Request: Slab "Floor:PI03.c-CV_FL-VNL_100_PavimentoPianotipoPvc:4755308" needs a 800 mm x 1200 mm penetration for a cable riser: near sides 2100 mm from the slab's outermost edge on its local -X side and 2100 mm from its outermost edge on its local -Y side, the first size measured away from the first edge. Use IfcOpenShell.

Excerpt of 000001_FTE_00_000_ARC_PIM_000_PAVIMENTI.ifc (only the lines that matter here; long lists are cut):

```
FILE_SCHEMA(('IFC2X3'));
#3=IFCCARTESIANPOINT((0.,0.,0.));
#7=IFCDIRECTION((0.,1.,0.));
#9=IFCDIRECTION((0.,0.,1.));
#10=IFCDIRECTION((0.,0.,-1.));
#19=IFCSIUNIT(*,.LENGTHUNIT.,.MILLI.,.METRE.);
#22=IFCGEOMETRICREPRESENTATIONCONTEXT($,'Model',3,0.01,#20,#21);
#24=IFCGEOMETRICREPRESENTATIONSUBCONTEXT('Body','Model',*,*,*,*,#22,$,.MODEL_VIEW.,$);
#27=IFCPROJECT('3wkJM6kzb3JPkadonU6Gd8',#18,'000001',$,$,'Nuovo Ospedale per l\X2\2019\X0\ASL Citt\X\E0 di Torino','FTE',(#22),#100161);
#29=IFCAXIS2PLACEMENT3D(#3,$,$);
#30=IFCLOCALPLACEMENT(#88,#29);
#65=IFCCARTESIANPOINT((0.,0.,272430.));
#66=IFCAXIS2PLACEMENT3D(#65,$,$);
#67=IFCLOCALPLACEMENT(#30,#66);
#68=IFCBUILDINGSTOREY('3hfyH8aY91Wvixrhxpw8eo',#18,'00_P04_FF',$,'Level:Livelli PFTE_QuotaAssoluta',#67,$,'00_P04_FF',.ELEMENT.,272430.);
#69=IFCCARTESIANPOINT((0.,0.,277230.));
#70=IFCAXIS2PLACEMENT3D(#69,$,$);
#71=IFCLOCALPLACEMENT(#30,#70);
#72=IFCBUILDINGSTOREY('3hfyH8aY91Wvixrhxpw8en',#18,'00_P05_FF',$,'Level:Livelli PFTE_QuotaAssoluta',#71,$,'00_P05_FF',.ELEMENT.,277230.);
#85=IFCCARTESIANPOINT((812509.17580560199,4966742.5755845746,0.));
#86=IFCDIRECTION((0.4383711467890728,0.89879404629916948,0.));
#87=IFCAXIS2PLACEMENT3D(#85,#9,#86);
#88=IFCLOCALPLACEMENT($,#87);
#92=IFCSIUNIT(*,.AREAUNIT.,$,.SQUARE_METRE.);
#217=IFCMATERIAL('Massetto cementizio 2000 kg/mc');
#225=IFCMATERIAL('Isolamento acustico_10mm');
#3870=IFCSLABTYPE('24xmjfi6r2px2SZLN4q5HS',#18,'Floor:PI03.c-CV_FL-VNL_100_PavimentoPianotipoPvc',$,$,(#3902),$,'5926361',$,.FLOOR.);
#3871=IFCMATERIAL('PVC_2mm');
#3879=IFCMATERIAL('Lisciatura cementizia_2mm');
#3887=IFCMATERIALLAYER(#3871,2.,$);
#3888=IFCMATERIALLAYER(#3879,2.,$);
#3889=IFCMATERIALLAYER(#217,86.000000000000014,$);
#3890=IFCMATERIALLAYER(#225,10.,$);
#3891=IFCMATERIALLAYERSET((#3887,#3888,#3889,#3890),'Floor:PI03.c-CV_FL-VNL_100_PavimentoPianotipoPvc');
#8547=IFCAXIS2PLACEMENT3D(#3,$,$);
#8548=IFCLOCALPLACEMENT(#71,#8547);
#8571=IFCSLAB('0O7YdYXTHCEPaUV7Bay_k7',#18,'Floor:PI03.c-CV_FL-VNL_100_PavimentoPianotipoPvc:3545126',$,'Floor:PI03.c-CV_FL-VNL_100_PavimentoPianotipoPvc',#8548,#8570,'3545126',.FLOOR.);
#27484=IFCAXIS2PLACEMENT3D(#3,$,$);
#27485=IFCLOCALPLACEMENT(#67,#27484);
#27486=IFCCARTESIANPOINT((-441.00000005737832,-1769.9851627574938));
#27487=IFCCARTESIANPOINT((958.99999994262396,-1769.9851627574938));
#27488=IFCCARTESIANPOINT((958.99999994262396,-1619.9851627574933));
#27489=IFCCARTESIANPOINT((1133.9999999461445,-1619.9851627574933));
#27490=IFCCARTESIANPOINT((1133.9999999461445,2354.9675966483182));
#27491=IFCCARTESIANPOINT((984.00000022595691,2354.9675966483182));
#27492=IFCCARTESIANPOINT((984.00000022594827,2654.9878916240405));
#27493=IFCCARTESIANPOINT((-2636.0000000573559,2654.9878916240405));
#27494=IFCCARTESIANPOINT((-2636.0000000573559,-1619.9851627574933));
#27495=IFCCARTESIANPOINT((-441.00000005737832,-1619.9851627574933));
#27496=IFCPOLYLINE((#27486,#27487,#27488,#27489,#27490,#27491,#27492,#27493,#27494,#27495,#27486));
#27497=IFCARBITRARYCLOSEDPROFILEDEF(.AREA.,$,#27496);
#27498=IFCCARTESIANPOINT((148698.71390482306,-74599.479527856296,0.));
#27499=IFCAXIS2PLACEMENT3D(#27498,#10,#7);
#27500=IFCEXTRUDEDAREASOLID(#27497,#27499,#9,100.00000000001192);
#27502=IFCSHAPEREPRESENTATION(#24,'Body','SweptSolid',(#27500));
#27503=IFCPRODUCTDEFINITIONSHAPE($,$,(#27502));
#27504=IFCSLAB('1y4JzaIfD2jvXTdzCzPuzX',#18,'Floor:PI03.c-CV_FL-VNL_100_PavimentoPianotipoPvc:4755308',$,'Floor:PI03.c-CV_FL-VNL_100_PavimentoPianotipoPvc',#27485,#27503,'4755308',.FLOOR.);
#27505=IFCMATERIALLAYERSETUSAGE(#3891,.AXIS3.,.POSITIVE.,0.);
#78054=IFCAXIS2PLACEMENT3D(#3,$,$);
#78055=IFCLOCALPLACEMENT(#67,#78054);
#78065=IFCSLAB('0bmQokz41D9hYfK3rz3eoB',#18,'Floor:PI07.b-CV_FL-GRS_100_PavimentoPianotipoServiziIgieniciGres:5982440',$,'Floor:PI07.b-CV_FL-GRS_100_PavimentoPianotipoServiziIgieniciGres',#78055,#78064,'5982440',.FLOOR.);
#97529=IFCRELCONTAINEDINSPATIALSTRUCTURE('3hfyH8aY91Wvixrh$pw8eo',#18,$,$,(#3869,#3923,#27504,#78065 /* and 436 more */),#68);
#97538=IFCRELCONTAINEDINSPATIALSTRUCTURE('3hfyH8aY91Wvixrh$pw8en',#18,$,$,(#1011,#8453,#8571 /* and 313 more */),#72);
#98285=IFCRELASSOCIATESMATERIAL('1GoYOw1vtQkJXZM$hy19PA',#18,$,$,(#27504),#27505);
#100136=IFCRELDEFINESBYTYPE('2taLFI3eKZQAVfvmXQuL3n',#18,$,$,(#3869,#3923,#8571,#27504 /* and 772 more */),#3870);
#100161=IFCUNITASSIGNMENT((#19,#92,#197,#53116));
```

```python
import numpy as np
import ifcopenshell
import ifcopenshell.api.feature
import ifcopenshell.api.geometry
import ifcopenshell.api.root
import ifcopenshell.geom
import ifcopenshell.util.placement
import ifcopenshell.util.representation
import ifcopenshell.util.shape
import ifcopenshell.util.unit

model = ifcopenshell.open("000001_FTE_00_000_ARC_PIM_000_PAVIMENTI.ifc")
unit_scale = ifcopenshell.util.unit.calculate_unit_scale(model)
settings = ifcopenshell.geom.settings()


def volume(element):
    """Net volume in cubic metres, openings subtracted."""
    shape = ifcopenshell.geom.create_shape(settings, element)
    return ifcopenshell.util.shape.get_volume(shape.geometry)


slab = model.by_guid("1y4JzaIfD2jvXTdzCzPuzX")
before = volume(slab)

# Extent in the slab's own axes, in metres. The edges named are its -X and -Y sides.
slab_shape = ifcopenshell.geom.create_shape(settings, slab)
vertices = ifcopenshell.util.shape.get_vertices(slab_shape.geometry)
x_min, y_min, bottom = vertices.min(axis=0)
top = vertices[:, 2].max()

opening = ifcopenshell.api.root.create_entity(model, ifc_class="IfcOpeningElement", name="Cable riser opening")
context = ifcopenshell.util.representation.get_context(model, "Model", "Body", "MODEL_VIEW")
width, depth = 0.8, 1.2
outline = [(0.0, 0.0), (width, 0.0), (width, depth), (0.0, depth), (0.0, 0.0)]
# Overshoot both faces by 50 mm so the cut is clean.
shape = ifcopenshell.api.geometry.add_slab_representation(
    model, context=context, depth=top - bottom + 0.1, polyline=outline
)
ifcopenshell.api.geometry.assign_representation(model, product=opening, representation=shape)

matrix = ifcopenshell.util.placement.get_local_placement(slab.ObjectPlacement)
matrix[:, 3] = matrix @ np.append(np.array([x_min + 2.1, y_min + 2.1, bottom - 0.05]) / unit_scale, 1.0)
ifcopenshell.api.geometry.edit_object_placement(model, product=opening, matrix=matrix, is_si=False)
ifcopenshell.api.feature.add_feature(model, feature=opening, element=slab)

after = volume(slab)

print(f"slab volume {before:.3f} -> {after:.3f} m3")

model.write("000001_FTE_00_000_ARC_PIM_000_PAVIMENTI-out.ifc")
```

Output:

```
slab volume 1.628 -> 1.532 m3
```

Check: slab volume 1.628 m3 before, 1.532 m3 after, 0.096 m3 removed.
